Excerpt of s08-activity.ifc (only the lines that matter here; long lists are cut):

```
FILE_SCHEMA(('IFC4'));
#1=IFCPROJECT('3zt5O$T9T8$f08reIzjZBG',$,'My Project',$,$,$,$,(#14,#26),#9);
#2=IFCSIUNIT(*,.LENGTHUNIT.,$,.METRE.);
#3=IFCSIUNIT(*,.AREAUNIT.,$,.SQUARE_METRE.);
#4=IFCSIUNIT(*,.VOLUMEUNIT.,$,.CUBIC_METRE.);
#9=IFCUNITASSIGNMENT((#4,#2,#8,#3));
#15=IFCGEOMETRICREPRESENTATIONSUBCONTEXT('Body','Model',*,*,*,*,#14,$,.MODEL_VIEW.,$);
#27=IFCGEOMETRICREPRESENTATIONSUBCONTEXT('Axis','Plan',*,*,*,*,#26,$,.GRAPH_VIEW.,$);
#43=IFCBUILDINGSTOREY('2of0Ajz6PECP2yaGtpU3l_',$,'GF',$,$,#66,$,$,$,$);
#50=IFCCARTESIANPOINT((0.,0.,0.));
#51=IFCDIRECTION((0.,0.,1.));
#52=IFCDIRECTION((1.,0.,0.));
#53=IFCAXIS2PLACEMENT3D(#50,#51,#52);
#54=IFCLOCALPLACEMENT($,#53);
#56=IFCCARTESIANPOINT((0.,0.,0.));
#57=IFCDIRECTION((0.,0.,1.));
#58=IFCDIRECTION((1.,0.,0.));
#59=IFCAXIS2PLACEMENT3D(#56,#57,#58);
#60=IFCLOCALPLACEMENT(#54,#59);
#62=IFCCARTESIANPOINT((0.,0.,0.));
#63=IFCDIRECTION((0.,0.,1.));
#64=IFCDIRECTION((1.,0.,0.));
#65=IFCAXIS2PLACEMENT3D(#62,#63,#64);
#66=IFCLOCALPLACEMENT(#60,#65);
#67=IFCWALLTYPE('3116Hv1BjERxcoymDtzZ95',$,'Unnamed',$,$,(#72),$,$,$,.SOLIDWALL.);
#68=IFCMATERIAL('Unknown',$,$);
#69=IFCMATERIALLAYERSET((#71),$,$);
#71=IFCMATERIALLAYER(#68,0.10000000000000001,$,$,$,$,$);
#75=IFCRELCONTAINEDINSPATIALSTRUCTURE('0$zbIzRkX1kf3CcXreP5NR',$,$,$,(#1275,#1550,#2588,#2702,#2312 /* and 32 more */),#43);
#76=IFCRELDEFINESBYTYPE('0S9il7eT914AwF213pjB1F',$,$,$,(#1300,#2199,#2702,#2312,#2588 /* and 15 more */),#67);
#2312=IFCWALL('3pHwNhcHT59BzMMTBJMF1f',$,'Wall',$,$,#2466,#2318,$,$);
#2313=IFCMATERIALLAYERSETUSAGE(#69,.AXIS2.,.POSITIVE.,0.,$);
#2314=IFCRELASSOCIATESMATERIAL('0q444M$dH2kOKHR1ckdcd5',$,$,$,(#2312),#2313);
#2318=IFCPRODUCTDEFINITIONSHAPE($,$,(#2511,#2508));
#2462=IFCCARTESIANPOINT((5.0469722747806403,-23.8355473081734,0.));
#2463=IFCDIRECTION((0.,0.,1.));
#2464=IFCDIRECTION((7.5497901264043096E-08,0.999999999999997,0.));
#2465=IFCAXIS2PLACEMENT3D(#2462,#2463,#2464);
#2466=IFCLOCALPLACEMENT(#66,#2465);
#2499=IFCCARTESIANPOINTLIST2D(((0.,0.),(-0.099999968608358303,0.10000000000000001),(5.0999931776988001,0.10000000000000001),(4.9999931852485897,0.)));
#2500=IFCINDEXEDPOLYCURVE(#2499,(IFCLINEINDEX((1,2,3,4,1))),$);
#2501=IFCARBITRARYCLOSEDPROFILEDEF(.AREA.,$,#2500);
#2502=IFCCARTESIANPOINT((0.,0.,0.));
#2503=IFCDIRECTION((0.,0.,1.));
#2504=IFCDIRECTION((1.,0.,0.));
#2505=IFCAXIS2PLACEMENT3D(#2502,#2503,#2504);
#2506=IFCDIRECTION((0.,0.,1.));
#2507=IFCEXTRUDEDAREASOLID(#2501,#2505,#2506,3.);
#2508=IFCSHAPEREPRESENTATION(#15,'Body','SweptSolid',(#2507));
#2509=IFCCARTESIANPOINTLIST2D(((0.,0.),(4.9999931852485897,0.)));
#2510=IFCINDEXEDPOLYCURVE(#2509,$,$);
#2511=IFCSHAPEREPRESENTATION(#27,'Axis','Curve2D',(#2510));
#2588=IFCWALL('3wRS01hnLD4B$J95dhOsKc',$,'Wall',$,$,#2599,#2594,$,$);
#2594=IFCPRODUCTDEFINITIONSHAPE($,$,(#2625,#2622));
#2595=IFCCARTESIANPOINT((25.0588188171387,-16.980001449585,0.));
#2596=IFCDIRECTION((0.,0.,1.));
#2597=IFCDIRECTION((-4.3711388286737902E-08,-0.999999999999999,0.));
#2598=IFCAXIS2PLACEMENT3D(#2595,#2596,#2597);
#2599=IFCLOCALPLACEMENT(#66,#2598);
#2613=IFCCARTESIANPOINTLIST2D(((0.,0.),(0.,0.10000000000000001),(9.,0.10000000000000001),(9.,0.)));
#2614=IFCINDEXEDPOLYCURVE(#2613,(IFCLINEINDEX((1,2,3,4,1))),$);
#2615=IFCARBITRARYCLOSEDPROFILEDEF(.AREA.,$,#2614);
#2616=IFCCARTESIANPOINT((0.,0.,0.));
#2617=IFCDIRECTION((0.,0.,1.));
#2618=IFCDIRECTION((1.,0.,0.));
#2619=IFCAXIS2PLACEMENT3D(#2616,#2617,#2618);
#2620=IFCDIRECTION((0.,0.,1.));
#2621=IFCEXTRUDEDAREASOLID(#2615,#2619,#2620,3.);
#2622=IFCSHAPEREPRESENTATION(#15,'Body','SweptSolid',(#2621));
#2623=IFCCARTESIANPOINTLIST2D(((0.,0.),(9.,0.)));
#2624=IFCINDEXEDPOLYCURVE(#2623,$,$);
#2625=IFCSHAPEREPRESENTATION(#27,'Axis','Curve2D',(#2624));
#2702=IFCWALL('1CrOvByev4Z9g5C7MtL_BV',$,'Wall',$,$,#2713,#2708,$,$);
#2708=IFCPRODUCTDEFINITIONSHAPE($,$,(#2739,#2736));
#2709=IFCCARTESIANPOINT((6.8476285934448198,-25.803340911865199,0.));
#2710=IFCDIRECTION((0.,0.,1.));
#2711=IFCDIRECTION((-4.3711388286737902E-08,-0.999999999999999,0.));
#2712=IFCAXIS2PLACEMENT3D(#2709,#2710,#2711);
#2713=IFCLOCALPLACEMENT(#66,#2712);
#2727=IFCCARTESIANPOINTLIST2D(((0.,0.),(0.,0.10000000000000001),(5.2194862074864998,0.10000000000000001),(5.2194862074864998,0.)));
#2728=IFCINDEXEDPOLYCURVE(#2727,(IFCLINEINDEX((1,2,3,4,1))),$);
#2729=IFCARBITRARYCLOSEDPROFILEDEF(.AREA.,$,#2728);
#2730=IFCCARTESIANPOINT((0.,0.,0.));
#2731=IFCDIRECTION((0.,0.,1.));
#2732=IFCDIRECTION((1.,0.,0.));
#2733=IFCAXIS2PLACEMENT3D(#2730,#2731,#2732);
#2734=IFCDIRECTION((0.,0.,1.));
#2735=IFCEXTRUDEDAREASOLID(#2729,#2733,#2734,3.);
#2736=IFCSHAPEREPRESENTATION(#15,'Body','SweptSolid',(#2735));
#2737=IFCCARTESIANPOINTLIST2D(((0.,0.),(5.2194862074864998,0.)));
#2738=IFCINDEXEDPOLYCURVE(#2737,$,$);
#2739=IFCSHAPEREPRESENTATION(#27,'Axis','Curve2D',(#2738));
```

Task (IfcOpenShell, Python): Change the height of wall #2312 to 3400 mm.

```python
import ifcopenshell
import ifcopenshell.geom
import ifcopenshell.util.representation
import ifcopenshell.util.shape

model = ifcopenshell.open("s08-activity.ifc")
settings = ifcopenshell.geom.settings()


def volume(element):
    """Net volume in cubic metres, openings subtracted."""
    shape = ifcopenshell.geom.create_shape(settings, element)
    return ifcopenshell.util.shape.get_volume(shape.geometry)


wall = model.by_guid("3pHwNhcHT59BzMMTBJMF1f")
before = volume(wall)

body = ifcopenshell.util.representation.get_representation(wall, "Model", "Body")
solid = body.Items[0]
old_height = solid.Depth
solid.Depth = 3.4
after = volume(wall)

print(f"height {old_height:g} -> {solid.Depth:g}, volume {before:.3f} -> {after:.3f} m3")

model.write("s08-activity_v2.ifc")
```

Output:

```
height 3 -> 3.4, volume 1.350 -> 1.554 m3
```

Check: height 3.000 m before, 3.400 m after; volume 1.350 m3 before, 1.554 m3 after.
